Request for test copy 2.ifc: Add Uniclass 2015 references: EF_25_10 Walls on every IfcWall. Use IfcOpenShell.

First a look at what the model holds.

```python
import ifcopenshell

model = ifcopenshell.open("test copy 2.ifc")
print(model.schema)
print("classifications:", [c.Name for c in model.by_type("IfcClassification")])
for ifc_class in ("IfcDoor", "IfcRoof", "IfcStair", "IfcWall", "IfcWindow"):
    print(ifc_class, len(model.by_type(ifc_class)))
```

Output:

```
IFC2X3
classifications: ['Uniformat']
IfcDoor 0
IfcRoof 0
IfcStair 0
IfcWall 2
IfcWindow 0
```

```python
import ifcopenshell
import ifcopenshell.api.classification

model = ifcopenshell.open("test copy 2.ifc")

# IFC2X3 requires Source and Edition and has no link from the project to the system.
system = model.create_entity("IfcClassification", Source="NBS", Edition="2015", Name="Uniclass 2015")

codes = {
    "IfcWall": ("EF_25_10", "Walls"),
}
for ifc_class, (code, name) in codes.items():
    products = model.by_type(ifc_class)
    ifcopenshell.api.classification.add_reference(
        model, products=products, classification=system, identification=code, name=name
    )
    print(code, len(products))

model.write("test copy 2_updated.ifc")
```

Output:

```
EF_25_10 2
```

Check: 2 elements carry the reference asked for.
